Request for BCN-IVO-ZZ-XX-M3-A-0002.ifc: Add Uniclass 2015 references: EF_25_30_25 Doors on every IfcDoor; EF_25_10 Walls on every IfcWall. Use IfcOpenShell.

First a look at what the model holds.

```python
import ifcopenshell

model = ifcopenshell.open("BCN-IVO-ZZ-XX-M3-A-0002.ifc")
print(model.schema)
print("classifications:", [c.Name for c in model.by_type("IfcClassification")])
for ifc_class in ("IfcDoor", "IfcRoof", "IfcStair", "IfcWall", "IfcWindow"):
    print(ifc_class, len(model.by_type(ifc_class)))
```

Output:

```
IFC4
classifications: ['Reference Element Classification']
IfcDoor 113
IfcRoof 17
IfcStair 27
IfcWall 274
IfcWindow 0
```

```python
import ifcopenshell
import ifcopenshell.api.classification

model = ifcopenshell.open("BCN-IVO-ZZ-XX-M3-A-0002.ifc")

system = ifcopenshell.api.classification.add_classification(model, classification="Uniclass 2015")

codes = {
    "IfcDoor": ("EF_25_30_25", "Doors"),
    "IfcWall": ("EF_25_10", "Walls"),
}
for ifc_class, (code, name) in codes.items():
    products = model.by_type(ifc_class)
    ifcopenshell.api.classification.add_reference(
        model, products=products, classification=system, identification=code, name=name
    )
    print(code, len(products))

model.write("BCN-IVO-ZZ-XX-M3-A-0002_rev.ifc")
```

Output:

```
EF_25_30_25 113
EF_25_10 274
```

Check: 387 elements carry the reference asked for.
